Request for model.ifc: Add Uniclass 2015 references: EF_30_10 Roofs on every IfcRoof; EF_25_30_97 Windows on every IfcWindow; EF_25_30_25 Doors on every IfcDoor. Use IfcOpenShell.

First a look at what the model holds.

```python
import ifcopenshell

model = ifcopenshell.open("model.ifc")
print(model.schema)
print("classifications:", [c.Name for c in model.by_type("IfcClassification")])
for ifc_class in ("IfcDoor", "IfcRoof", "IfcStair", "IfcWall", "IfcWindow"):
    print(ifc_class, len(model.by_type(ifc_class)))
```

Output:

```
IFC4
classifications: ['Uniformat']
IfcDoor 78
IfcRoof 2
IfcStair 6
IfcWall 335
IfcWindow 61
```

```python
import ifcopenshell
import ifcopenshell.api.classification

model = ifcopenshell.open("model.ifc")

system = ifcopenshell.api.classification.add_classification(model, classification="Uniclass 2015")

codes = {
    "IfcRoof": ("EF_30_10", "Roofs"),
    "IfcWindow": ("EF_25_30_97", "Windows"),
    "IfcDoor": ("EF_25_30_25", "Doors"),
}
for ifc_class, (code, name) in codes.items():
    products = model.by_type(ifc_class)
    ifcopenshell.api.classification.add_reference(
        model, products=products, classification=system, identification=code, name=name
    )
    print(code, len(products))

model.write("model_rev.ifc")
```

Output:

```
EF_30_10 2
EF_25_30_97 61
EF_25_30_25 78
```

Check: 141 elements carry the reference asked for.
